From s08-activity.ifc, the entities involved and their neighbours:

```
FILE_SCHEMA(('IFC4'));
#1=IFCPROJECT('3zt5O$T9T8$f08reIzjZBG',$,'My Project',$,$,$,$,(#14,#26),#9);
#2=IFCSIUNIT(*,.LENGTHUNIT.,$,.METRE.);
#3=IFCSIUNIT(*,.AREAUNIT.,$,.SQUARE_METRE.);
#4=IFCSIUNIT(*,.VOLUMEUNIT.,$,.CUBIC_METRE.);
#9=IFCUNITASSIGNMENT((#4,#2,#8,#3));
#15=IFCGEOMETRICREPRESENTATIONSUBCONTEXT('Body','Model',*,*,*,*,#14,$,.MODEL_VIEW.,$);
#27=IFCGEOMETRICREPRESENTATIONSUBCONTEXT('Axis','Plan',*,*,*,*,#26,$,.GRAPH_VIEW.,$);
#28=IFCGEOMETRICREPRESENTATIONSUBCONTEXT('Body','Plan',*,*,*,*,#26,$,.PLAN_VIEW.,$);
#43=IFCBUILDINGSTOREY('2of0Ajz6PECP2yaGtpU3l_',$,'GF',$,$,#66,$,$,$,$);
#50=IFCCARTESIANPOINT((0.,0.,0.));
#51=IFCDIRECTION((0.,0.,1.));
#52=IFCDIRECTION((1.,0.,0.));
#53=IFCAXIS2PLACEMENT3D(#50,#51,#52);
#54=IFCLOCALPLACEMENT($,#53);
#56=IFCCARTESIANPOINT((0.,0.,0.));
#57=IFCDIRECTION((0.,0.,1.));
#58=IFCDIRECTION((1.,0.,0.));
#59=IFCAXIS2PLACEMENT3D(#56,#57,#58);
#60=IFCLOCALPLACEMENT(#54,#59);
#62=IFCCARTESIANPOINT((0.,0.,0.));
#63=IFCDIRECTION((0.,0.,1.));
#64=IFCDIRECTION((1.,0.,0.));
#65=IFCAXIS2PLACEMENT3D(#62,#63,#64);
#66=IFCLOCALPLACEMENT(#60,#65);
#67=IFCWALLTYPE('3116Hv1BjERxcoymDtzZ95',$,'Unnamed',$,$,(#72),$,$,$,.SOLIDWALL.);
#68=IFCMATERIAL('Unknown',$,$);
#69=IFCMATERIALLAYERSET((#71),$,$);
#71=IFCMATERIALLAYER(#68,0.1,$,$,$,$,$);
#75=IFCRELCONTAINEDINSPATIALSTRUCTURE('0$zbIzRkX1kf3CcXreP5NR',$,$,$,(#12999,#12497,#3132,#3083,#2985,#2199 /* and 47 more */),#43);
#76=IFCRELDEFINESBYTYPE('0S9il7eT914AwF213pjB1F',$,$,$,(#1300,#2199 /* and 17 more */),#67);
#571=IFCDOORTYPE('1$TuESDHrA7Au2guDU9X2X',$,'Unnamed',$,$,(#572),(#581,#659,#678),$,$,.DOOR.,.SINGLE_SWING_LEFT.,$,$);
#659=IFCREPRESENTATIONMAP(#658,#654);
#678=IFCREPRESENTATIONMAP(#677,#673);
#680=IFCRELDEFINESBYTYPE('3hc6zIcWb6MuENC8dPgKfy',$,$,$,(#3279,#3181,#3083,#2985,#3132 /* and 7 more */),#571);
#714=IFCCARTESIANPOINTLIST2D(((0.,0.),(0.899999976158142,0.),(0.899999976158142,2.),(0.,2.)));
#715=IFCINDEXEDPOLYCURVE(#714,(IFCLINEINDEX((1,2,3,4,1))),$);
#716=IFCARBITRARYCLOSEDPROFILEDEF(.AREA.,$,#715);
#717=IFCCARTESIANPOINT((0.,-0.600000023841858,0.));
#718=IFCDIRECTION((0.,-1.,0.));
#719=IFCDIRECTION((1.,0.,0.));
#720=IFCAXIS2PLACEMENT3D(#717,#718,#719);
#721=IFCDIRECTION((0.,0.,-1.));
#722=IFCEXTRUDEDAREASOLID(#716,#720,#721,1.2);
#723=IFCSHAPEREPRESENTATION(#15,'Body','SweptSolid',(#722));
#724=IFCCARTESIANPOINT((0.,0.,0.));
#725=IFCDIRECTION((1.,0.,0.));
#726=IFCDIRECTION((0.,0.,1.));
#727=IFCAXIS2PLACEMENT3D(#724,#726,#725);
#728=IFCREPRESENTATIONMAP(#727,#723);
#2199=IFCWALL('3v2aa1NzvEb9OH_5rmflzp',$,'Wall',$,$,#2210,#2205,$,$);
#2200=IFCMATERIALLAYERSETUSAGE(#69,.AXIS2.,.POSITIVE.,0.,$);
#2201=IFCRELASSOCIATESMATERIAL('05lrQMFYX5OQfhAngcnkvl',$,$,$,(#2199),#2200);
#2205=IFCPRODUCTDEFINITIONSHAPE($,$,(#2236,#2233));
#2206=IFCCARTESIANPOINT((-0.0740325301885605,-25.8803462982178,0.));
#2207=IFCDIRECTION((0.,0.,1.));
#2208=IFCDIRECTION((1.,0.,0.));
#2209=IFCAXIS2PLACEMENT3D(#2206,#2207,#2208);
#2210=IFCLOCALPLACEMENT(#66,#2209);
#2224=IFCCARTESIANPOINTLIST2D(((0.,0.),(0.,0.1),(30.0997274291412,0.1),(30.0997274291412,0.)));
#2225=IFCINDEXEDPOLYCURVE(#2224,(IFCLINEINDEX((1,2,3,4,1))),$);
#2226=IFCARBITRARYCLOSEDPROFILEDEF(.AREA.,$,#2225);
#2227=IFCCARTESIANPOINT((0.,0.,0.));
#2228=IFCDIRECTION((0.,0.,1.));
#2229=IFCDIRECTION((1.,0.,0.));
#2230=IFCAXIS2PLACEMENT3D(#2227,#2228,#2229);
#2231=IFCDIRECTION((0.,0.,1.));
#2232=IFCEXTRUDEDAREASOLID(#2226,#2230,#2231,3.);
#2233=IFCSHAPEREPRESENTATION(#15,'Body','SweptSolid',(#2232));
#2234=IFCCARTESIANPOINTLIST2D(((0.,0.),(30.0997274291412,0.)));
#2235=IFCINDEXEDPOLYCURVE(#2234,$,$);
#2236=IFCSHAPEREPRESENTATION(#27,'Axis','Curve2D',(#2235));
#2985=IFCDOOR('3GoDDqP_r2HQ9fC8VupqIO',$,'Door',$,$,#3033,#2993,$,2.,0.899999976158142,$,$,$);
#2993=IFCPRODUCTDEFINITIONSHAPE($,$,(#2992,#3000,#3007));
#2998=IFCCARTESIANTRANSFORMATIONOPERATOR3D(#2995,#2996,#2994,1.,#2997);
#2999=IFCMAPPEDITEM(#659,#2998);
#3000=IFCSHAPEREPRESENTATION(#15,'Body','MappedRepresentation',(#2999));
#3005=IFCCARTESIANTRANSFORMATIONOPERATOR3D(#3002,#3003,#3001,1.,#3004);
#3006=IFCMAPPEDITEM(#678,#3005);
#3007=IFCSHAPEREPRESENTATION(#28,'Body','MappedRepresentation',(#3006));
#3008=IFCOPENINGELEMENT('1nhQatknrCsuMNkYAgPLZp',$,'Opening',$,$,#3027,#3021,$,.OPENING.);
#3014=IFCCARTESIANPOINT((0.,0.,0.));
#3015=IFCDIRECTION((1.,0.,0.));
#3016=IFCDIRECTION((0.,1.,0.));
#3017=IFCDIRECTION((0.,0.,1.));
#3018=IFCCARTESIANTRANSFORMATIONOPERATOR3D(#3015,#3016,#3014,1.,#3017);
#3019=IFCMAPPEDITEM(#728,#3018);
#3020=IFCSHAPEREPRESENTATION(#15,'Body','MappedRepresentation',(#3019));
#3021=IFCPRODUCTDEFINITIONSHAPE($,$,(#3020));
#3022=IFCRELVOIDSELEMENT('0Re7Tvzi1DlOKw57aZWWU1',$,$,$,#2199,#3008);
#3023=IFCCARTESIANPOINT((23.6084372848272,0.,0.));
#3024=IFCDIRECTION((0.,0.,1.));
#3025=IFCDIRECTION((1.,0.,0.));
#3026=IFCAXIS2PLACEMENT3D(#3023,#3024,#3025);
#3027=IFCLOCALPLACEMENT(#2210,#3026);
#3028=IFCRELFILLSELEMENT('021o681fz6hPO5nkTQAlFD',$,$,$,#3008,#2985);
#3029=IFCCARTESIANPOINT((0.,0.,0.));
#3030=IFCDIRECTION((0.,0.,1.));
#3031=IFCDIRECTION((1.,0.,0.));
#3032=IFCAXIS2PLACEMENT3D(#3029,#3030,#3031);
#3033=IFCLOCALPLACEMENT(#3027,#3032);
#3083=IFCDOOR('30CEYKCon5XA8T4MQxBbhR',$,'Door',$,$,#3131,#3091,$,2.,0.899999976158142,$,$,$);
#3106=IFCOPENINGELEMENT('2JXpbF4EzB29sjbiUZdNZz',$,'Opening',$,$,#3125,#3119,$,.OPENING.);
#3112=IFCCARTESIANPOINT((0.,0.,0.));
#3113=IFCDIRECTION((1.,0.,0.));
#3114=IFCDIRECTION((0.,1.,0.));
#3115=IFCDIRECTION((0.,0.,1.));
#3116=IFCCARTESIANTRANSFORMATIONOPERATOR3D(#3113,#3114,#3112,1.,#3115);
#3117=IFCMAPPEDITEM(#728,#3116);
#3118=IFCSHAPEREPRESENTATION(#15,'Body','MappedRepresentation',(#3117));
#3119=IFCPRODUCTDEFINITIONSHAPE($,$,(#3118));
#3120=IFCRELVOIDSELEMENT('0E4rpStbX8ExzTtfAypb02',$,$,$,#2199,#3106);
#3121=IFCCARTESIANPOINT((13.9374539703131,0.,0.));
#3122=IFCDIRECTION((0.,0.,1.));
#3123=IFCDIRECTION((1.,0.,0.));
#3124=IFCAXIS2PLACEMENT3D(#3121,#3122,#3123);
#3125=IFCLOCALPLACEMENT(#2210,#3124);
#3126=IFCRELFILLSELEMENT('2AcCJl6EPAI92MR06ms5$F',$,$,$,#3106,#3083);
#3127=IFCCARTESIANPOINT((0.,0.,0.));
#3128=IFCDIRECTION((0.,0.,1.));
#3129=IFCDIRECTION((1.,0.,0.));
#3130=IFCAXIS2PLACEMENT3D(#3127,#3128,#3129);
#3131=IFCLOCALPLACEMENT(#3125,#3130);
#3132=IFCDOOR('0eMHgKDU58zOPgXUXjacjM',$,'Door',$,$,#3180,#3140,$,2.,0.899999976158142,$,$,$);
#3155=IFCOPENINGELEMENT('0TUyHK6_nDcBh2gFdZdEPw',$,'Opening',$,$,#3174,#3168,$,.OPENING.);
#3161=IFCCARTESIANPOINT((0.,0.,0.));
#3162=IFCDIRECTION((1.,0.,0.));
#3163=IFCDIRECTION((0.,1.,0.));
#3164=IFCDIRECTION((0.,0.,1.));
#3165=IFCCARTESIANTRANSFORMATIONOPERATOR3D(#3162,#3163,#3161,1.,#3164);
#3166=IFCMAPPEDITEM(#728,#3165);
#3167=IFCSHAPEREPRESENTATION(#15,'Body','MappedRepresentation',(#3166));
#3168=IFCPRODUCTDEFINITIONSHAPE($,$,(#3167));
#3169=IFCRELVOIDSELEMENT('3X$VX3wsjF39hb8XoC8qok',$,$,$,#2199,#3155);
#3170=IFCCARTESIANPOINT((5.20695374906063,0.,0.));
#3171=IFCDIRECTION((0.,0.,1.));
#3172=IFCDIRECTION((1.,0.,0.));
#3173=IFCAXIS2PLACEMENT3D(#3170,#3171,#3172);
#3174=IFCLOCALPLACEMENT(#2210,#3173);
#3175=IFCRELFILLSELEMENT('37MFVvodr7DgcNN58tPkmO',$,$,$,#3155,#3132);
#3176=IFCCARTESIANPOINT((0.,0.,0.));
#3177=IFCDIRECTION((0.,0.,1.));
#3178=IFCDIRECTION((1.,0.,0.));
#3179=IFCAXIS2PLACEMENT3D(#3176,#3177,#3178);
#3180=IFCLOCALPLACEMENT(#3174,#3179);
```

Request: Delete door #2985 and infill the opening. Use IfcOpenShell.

```python
import ifcopenshell
import ifcopenshell.api.feature
import ifcopenshell.api.root
import ifcopenshell.geom
import ifcopenshell.util.shape

model = ifcopenshell.open("s08-activity.ifc")
settings = ifcopenshell.geom.settings()


def volume(element):
    """Net volume in cubic metres, openings subtracted."""
    shape = ifcopenshell.geom.create_shape(settings, element)
    return ifcopenshell.util.shape.get_volume(shape.geometry)


door = model.by_guid("3GoDDqP_r2HQ9fC8VupqIO")
opening = door.FillsVoids[0].RelatingOpeningElement
wall = opening.VoidsElements[0].RelatingBuildingElement
before = volume(wall)

ifcopenshell.api.root.remove_product(model, product=door)
ifcopenshell.api.feature.remove_feature(model, feature=opening)

after = volume(wall)

print(f"wall volume {before:.3f} -> {after:.3f} m3")

model.write("s08-activity_edited.ifc")
```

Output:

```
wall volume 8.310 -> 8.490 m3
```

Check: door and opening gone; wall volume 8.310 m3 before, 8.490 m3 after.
